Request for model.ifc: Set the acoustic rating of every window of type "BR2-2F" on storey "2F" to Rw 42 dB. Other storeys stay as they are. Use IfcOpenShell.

First a look at what the model holds.

```python
import ifcopenshell
import ifcopenshell.util.element

model = ifcopenshell.open("model.ifc")
print(model.schema)
storey = next(s for s in model.by_type("IfcBuildingStorey") if s.Name == "2F")
windows = [e for e in ifcopenshell.util.element.get_decomposition(storey) if e.is_a("IfcWindow")]
seen = {}
for e in windows:
    element_type = ifcopenshell.util.element.get_type(e)
    key = (element_type.Name if element_type != e and element_type else None, ifcopenshell.util.element.get_pset(e, "Pset_WindowCommon", "AcousticRating"))
    seen[key] = seen.get(key, 0) + 1
for (name, value), count in sorted(seen.items(), key=str):
    print(count, "x", name, "|", value)
```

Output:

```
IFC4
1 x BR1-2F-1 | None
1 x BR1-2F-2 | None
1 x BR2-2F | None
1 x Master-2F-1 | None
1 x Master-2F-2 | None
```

```python
import ifcopenshell
import ifcopenshell.api.pset
import ifcopenshell.util.element

model = ifcopenshell.open("model.ifc")

storey = next(s for s in model.by_type("IfcBuildingStorey") if s.Name == "2F")
windows = [e for e in ifcopenshell.util.element.get_decomposition(storey) if e.is_a("IfcWindow")]

count = 0
for e in windows:
    element_type = ifcopenshell.util.element.get_type(e)
    if element_type in (None, e) or element_type.Name != "BR2-2F":
        continue
    # add_pset returns the element's existing set when there is one.
    pset = ifcopenshell.api.pset.add_pset(model, product=e, name="Pset_WindowCommon")
    ifcopenshell.api.pset.edit_pset(model, pset=pset, properties={"AcousticRating": "Rw 42 dB"})
    count += 1

print(count, "windows updated")

model.write("model_edited.ifc")
```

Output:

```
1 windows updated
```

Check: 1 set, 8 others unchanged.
